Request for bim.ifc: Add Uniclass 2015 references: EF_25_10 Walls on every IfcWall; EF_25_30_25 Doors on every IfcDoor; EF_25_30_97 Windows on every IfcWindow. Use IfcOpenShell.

First a look at what the model holds.

```python
import ifcopenshell

model = ifcopenshell.open("bim.ifc")
print(model.schema)
print("classifications:", [c.Name for c in model.by_type("IfcClassification")])
for ifc_class in ("IfcDoor", "IfcRoof", "IfcStair", "IfcWall", "IfcWindow"):
    print(ifc_class, len(model.by_type(ifc_class)))
```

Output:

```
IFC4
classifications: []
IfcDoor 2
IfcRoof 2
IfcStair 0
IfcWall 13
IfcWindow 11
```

```python
import ifcopenshell
import ifcopenshell.api.classification

model = ifcopenshell.open("bim.ifc")

system = ifcopenshell.api.classification.add_classification(model, classification="Uniclass 2015")

codes = {
    "IfcWall": ("EF_25_10", "Walls"),
    "IfcDoor": ("EF_25_30_25", "Doors"),
    "IfcWindow": ("EF_25_30_97", "Windows"),
}
for ifc_class, (code, name) in codes.items():
    products = model.by_type(ifc_class)
    ifcopenshell.api.classification.add_reference(
        model, products=products, classification=system, identification=code, name=name
    )
    print(code, len(products))

model.write("bim_rev.ifc")
```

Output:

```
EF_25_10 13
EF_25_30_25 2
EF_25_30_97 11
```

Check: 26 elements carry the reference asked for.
